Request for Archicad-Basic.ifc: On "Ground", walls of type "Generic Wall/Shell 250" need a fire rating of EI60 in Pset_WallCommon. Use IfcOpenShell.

First a look at what the model holds.

```python
import ifcopenshell
import ifcopenshell.util.element

model = ifcopenshell.open("Archicad-Basic.ifc")
print(model.schema)
storey = next(s for s in model.by_type("IfcBuildingStorey") if s.Name == "Ground")
walls = [e for e in ifcopenshell.util.element.get_decomposition(storey) if e.is_a("IfcWall")]
seen = {}
for e in walls:
    element_type = ifcopenshell.util.element.get_type(e)
    key = (element_type.Name if element_type != e and element_type else None, ifcopenshell.util.element.get_pset(e, "Pset_WallCommon", "FireRating"))
    seen[key] = seen.get(key, 0) + 1
for (name, value), count in sorted(seen.items(), key=str):
    print(count, "x", name, "|", value)
```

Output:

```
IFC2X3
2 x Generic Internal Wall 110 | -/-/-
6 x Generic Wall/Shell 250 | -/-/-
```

```python
import ifcopenshell
import ifcopenshell.api.pset
import ifcopenshell.util.element

model = ifcopenshell.open("Archicad-Basic.ifc")

storey = next(s for s in model.by_type("IfcBuildingStorey") if s.Name == "Ground")
walls = [e for e in ifcopenshell.util.element.get_decomposition(storey) if e.is_a("IfcWall")]

count = 0
for e in walls:
    element_type = ifcopenshell.util.element.get_type(e)
    if element_type in (None, e) or element_type.Name != "Generic Wall/Shell 250":
        continue
    # add_pset returns the element's existing set when there is one.
    pset = ifcopenshell.api.pset.add_pset(model, product=e, name="Pset_WallCommon")
    ifcopenshell.api.pset.edit_pset(model, pset=pset, properties={"FireRating": "EI60"})
    count += 1

print(count, "walls updated")

model.write("Archicad-Basic_updated.ifc")
```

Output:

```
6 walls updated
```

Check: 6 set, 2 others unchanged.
